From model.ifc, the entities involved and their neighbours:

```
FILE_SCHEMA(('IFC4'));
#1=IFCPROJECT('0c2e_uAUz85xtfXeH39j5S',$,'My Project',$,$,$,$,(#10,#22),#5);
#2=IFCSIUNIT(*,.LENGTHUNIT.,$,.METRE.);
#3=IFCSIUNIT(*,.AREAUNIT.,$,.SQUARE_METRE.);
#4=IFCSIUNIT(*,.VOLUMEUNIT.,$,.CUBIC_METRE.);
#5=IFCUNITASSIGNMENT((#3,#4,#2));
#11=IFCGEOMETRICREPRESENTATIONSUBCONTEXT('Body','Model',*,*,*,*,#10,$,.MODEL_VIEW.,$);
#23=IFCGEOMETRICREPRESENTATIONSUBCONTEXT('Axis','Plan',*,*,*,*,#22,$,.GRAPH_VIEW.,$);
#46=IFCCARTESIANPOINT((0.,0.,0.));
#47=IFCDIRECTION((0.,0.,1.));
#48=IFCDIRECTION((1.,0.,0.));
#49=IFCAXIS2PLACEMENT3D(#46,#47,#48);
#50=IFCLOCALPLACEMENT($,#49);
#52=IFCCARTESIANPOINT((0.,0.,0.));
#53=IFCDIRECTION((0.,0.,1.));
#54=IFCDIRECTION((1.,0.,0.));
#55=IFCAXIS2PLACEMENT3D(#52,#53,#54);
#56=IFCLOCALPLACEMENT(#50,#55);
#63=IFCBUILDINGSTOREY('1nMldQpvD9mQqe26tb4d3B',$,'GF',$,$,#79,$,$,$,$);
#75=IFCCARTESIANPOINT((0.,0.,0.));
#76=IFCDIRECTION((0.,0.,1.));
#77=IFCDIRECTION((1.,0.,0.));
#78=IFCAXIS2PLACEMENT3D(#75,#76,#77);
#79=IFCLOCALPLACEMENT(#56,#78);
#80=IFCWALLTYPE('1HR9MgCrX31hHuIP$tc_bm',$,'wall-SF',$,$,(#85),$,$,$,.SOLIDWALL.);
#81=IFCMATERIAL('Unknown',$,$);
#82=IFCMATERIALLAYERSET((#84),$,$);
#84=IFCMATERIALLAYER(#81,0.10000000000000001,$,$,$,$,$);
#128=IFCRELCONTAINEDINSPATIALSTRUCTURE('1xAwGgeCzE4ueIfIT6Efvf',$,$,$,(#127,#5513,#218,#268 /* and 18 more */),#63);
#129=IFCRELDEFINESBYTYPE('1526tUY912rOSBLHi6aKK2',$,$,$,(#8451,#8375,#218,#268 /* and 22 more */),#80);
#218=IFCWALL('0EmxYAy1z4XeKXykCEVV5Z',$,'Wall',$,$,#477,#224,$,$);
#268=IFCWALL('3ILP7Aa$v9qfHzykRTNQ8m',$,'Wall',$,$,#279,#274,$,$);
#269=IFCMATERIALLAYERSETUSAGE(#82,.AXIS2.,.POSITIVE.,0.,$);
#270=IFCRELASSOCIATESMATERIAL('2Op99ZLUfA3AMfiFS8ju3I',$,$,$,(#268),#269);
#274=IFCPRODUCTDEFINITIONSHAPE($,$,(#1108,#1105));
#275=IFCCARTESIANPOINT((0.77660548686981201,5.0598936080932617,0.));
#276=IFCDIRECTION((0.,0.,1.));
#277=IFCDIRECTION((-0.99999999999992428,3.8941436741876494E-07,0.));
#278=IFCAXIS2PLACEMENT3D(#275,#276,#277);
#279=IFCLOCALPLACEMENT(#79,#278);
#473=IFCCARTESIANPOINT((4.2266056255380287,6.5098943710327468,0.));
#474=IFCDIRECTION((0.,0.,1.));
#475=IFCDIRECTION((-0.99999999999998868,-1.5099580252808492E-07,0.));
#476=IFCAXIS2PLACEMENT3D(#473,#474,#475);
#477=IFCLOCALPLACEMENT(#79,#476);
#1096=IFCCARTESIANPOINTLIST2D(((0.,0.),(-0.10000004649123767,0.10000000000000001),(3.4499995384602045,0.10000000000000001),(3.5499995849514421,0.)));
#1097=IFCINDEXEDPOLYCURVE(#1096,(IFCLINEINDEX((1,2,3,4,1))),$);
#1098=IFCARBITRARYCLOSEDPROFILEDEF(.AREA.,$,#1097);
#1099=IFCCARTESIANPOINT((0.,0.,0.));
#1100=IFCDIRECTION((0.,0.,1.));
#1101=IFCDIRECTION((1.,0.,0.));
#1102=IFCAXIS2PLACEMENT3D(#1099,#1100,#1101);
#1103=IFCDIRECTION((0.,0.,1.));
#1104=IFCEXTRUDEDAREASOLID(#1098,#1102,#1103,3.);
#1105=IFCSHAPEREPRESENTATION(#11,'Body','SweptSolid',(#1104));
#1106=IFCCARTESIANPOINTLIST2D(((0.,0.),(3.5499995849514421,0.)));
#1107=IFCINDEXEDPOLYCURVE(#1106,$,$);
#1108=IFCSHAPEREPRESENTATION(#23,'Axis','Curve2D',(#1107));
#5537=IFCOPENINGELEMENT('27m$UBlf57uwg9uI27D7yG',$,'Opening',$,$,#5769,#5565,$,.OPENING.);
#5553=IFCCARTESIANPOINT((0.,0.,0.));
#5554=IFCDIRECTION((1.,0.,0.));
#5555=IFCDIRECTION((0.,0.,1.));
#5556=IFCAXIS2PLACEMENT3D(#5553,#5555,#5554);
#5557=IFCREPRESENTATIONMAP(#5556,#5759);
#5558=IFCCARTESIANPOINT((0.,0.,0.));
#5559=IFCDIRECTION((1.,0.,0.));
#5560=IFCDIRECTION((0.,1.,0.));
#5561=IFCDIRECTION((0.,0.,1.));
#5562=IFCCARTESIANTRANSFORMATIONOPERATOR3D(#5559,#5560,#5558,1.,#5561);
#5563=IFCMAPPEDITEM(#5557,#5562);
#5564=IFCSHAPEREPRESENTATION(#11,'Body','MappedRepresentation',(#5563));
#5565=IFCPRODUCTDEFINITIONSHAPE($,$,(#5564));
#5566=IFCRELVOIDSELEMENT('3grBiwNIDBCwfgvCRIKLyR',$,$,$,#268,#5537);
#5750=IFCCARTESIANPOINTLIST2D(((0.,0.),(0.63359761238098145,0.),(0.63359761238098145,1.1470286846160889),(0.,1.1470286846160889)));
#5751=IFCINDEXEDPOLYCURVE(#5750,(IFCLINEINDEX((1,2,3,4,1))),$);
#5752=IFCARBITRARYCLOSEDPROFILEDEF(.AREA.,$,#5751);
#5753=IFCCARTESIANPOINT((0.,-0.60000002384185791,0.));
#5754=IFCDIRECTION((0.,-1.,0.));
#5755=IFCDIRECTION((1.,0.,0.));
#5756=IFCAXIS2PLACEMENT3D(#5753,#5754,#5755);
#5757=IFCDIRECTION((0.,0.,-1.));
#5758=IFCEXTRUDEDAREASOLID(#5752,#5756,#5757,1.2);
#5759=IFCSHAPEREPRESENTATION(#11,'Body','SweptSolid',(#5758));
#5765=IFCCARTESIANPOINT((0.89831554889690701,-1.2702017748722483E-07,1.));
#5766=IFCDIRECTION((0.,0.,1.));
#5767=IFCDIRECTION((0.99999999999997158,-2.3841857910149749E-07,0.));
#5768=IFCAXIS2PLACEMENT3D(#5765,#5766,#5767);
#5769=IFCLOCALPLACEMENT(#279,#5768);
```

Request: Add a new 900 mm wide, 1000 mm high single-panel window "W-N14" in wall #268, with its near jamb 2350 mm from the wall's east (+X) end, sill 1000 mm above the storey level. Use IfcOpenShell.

```python
import numpy as np
import ifcopenshell
import ifcopenshell.api.feature
import ifcopenshell.api.geometry
import ifcopenshell.api.root
import ifcopenshell.api.spatial
import ifcopenshell.geom
import ifcopenshell.util.element
import ifcopenshell.util.placement
import ifcopenshell.util.representation
import ifcopenshell.util.shape
import ifcopenshell.util.unit

model = ifcopenshell.open("model.ifc")
unit_scale = ifcopenshell.util.unit.calculate_unit_scale(model)
settings = ifcopenshell.geom.settings()


def volume(element):
    """Net volume in cubic metres, openings subtracted."""
    shape = ifcopenshell.geom.create_shape(settings, element)
    return ifcopenshell.util.shape.get_volume(shape.geometry)


wall = model.by_guid("3ILP7Aa$v9qfHzykRTNQ8m")
storey = ifcopenshell.util.element.get_container(wall, ifc_class="IfcBuildingStorey")
context = ifcopenshell.util.representation.get_context(model, "Model", "Body", "MODEL_VIEW")
before = volume(wall)

width, height, from_end, sill = 0.9, 1, 2.35, 1  # metres

# The wall runs along its own X axis, and the end named is its -X end.
wall_shape = ifcopenshell.geom.create_shape(settings, wall)
x, y, z = ifcopenshell.util.shape.get_vertices(wall_shape.geometry).T
start = x.min() + from_end
face, thickness = float(y.min()), float(y.max() - y.min())
wall_matrix = ifcopenshell.util.placement.get_local_placement(wall.ObjectPlacement)
level = ifcopenshell.util.placement.get_local_placement(storey.ObjectPlacement)[2, 3]


def in_wall(x, y):
    """Placement at x, y metres in the wall's axes, at sill height."""
    matrix = wall_matrix.copy()
    matrix[:, 3] = wall_matrix @ np.array([x / unit_scale, y / unit_scale, 0.0, 1.0])
    matrix[2, 3] = level + sill / unit_scale
    return matrix


# Opening: a box that overshoots both wall faces by 50 mm.
opening = ifcopenshell.api.root.create_entity(model, ifc_class="IfcOpeningElement", predefined_type="OPENING")
box = ifcopenshell.api.geometry.add_wall_representation(
    model, context=context, length=width, height=height, thickness=thickness + 0.1
)
ifcopenshell.api.geometry.assign_representation(model, product=opening, representation=box)
ifcopenshell.api.geometry.edit_object_placement(model, product=opening, matrix=in_wall(start, face - 0.05), is_si=False)
ifcopenshell.api.feature.add_feature(model, feature=opening, element=wall)

window = ifcopenshell.api.root.create_entity(model, ifc_class="IfcWindow", name="W-N14", predefined_type="WINDOW")
window.OverallWidth, window.OverallHeight = width / unit_scale, height / unit_scale
window.PartitioningType = "SINGLE_PANEL"
body = ifcopenshell.api.geometry.add_window_representation(
    model,
    context=context,
    overall_width=window.OverallWidth,
    overall_height=window.OverallHeight,
    partition_type="SINGLE_PANEL",
)
ifcopenshell.api.geometry.assign_representation(model, product=window, representation=body)
ifcopenshell.api.spatial.assign_container(model, products=[window], relating_structure=storey)
ifcopenshell.api.feature.add_filling(model, opening=opening, element=window)

# Centre the window in the wall's thickness.
ifcopenshell.api.geometry.edit_object_placement(model, product=window, matrix=in_wall(start, face), is_si=False)
window_shape = ifcopenshell.geom.create_shape(settings, window)
depth = ifcopenshell.util.shape.get_vertices(window_shape.geometry)[:, 1]
offset = face + thickness / 2 - (depth.min() + depth.max()) / 2
ifcopenshell.api.geometry.edit_object_placement(model, product=window, matrix=in_wall(start, offset), is_si=False)

after = volume(wall)

print(f"wall volume {before:.3f} -> {after:.3f} m3")

model.write("model_rev.ifc")
```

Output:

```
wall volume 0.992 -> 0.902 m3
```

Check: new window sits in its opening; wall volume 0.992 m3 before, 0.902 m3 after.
